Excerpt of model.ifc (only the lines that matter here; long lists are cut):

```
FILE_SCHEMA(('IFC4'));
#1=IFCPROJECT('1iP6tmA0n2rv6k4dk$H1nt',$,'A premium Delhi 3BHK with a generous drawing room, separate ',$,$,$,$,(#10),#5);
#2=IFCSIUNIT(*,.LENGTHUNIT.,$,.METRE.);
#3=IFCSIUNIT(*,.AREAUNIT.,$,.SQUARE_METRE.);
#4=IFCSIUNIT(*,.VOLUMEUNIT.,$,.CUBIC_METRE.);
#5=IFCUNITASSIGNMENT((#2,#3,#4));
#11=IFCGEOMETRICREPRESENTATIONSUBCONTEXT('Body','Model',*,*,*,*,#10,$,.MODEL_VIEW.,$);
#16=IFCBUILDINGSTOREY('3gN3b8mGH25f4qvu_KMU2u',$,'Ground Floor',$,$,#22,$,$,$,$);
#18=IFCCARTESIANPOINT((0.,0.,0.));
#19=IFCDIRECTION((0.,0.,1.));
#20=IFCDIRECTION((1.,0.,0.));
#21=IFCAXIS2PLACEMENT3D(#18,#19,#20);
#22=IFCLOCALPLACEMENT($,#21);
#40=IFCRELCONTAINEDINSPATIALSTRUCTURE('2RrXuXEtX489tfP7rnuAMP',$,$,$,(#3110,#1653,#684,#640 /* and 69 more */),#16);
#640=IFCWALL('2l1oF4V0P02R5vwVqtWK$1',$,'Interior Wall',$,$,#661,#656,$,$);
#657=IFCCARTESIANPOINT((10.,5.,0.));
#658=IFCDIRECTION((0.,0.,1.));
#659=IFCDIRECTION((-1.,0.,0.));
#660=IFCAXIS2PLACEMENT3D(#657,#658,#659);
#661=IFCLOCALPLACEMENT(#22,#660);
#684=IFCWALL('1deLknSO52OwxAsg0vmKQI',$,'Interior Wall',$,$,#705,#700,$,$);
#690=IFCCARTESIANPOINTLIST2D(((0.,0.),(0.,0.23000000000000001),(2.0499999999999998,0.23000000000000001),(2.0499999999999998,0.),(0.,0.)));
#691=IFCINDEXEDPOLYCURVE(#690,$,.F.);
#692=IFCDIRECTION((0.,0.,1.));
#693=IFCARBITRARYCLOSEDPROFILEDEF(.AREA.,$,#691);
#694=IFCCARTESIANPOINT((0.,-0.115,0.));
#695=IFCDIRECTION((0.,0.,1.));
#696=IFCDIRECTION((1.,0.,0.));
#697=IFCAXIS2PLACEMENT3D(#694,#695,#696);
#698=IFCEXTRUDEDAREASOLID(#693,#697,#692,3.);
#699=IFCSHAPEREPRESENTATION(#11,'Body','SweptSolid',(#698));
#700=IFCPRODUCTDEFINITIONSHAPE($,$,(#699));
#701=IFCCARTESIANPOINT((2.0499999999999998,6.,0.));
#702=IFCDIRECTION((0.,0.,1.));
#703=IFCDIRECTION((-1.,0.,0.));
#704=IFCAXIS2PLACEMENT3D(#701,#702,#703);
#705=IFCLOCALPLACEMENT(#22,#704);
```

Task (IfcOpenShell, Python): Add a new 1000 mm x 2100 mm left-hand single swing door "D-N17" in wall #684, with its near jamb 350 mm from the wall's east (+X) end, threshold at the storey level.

```python
import numpy as np
import ifcopenshell
import ifcopenshell.api.feature
import ifcopenshell.api.geometry
import ifcopenshell.api.root
import ifcopenshell.api.spatial
import ifcopenshell.geom
import ifcopenshell.util.element
import ifcopenshell.util.placement
import ifcopenshell.util.representation
import ifcopenshell.util.shape
import ifcopenshell.util.unit

model = ifcopenshell.open("model.ifc")
unit_scale = ifcopenshell.util.unit.calculate_unit_scale(model)
settings = ifcopenshell.geom.settings()


def volume(element):
    """Net volume in cubic metres, openings subtracted."""
    shape = ifcopenshell.geom.create_shape(settings, element)
    return ifcopenshell.util.shape.get_volume(shape.geometry)


wall = model.by_guid("1deLknSO52OwxAsg0vmKQI")
storey = ifcopenshell.util.element.get_container(wall, ifc_class="IfcBuildingStorey")
context = ifcopenshell.util.representation.get_context(model, "Model", "Body", "MODEL_VIEW")
before = volume(wall)

width, height, from_end, sill = 1, 2.1, 0.35, 0.0  # metres

# The wall runs along its own X axis, and the end named is its -X end.
wall_shape = ifcopenshell.geom.create_shape(settings, wall)
x, y, z = ifcopenshell.util.shape.get_vertices(wall_shape.geometry).T
start = x.min() + from_end
face, thickness = float(y.min()), float(y.max() - y.min())
wall_matrix = ifcopenshell.util.placement.get_local_placement(wall.ObjectPlacement)
level = ifcopenshell.util.placement.get_local_placement(storey.ObjectPlacement)[2, 3]


def in_wall(x, y):
    """Placement at x, y metres in the wall's axes, at sill height."""
    matrix = wall_matrix.copy()
    matrix[:, 3] = wall_matrix @ np.array([x / unit_scale, y / unit_scale, 0.0, 1.0])
    matrix[2, 3] = level + sill / unit_scale
    return matrix


# Opening: a box that overshoots both wall faces by 50 mm.
opening = ifcopenshell.api.root.create_entity(model, ifc_class="IfcOpeningElement", predefined_type="OPENING")
box = ifcopenshell.api.geometry.add_wall_representation(
    model, context=context, length=width, height=height, thickness=thickness + 0.1
)
ifcopenshell.api.geometry.assign_representation(model, product=opening, representation=box)
ifcopenshell.api.geometry.edit_object_placement(model, product=opening, matrix=in_wall(start, face - 0.05), is_si=False)
ifcopenshell.api.feature.add_feature(model, feature=opening, element=wall)

door = ifcopenshell.api.root.create_entity(model, ifc_class="IfcDoor", name="D-N17", predefined_type="DOOR")
door.OverallWidth, door.OverallHeight = width / unit_scale, height / unit_scale
door.OperationType = "SINGLE_SWING_LEFT"
body = ifcopenshell.api.geometry.add_door_representation(
    model,
    context=context,
    overall_width=door.OverallWidth,
    overall_height=door.OverallHeight,
    operation_type="SINGLE_SWING_LEFT",
    lining_properties={"LiningDepth": thickness / unit_scale, "ThresholdDepth": thickness / unit_scale},
)
ifcopenshell.api.geometry.assign_representation(model, product=door, representation=body)
ifcopenshell.api.spatial.assign_container(model, products=[door], relating_structure=storey)
ifcopenshell.api.feature.add_filling(model, opening=opening, element=door)

# The lining spans the wall, so the door starts at the wall face.
ifcopenshell.api.geometry.edit_object_placement(model, product=door, matrix=in_wall(start, face), is_si=False)

after = volume(wall)

print(f"wall volume {before:.3f} -> {after:.3f} m3")

model.write("model_rev.ifc")
```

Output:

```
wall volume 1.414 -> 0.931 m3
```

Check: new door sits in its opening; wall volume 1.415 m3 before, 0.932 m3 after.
